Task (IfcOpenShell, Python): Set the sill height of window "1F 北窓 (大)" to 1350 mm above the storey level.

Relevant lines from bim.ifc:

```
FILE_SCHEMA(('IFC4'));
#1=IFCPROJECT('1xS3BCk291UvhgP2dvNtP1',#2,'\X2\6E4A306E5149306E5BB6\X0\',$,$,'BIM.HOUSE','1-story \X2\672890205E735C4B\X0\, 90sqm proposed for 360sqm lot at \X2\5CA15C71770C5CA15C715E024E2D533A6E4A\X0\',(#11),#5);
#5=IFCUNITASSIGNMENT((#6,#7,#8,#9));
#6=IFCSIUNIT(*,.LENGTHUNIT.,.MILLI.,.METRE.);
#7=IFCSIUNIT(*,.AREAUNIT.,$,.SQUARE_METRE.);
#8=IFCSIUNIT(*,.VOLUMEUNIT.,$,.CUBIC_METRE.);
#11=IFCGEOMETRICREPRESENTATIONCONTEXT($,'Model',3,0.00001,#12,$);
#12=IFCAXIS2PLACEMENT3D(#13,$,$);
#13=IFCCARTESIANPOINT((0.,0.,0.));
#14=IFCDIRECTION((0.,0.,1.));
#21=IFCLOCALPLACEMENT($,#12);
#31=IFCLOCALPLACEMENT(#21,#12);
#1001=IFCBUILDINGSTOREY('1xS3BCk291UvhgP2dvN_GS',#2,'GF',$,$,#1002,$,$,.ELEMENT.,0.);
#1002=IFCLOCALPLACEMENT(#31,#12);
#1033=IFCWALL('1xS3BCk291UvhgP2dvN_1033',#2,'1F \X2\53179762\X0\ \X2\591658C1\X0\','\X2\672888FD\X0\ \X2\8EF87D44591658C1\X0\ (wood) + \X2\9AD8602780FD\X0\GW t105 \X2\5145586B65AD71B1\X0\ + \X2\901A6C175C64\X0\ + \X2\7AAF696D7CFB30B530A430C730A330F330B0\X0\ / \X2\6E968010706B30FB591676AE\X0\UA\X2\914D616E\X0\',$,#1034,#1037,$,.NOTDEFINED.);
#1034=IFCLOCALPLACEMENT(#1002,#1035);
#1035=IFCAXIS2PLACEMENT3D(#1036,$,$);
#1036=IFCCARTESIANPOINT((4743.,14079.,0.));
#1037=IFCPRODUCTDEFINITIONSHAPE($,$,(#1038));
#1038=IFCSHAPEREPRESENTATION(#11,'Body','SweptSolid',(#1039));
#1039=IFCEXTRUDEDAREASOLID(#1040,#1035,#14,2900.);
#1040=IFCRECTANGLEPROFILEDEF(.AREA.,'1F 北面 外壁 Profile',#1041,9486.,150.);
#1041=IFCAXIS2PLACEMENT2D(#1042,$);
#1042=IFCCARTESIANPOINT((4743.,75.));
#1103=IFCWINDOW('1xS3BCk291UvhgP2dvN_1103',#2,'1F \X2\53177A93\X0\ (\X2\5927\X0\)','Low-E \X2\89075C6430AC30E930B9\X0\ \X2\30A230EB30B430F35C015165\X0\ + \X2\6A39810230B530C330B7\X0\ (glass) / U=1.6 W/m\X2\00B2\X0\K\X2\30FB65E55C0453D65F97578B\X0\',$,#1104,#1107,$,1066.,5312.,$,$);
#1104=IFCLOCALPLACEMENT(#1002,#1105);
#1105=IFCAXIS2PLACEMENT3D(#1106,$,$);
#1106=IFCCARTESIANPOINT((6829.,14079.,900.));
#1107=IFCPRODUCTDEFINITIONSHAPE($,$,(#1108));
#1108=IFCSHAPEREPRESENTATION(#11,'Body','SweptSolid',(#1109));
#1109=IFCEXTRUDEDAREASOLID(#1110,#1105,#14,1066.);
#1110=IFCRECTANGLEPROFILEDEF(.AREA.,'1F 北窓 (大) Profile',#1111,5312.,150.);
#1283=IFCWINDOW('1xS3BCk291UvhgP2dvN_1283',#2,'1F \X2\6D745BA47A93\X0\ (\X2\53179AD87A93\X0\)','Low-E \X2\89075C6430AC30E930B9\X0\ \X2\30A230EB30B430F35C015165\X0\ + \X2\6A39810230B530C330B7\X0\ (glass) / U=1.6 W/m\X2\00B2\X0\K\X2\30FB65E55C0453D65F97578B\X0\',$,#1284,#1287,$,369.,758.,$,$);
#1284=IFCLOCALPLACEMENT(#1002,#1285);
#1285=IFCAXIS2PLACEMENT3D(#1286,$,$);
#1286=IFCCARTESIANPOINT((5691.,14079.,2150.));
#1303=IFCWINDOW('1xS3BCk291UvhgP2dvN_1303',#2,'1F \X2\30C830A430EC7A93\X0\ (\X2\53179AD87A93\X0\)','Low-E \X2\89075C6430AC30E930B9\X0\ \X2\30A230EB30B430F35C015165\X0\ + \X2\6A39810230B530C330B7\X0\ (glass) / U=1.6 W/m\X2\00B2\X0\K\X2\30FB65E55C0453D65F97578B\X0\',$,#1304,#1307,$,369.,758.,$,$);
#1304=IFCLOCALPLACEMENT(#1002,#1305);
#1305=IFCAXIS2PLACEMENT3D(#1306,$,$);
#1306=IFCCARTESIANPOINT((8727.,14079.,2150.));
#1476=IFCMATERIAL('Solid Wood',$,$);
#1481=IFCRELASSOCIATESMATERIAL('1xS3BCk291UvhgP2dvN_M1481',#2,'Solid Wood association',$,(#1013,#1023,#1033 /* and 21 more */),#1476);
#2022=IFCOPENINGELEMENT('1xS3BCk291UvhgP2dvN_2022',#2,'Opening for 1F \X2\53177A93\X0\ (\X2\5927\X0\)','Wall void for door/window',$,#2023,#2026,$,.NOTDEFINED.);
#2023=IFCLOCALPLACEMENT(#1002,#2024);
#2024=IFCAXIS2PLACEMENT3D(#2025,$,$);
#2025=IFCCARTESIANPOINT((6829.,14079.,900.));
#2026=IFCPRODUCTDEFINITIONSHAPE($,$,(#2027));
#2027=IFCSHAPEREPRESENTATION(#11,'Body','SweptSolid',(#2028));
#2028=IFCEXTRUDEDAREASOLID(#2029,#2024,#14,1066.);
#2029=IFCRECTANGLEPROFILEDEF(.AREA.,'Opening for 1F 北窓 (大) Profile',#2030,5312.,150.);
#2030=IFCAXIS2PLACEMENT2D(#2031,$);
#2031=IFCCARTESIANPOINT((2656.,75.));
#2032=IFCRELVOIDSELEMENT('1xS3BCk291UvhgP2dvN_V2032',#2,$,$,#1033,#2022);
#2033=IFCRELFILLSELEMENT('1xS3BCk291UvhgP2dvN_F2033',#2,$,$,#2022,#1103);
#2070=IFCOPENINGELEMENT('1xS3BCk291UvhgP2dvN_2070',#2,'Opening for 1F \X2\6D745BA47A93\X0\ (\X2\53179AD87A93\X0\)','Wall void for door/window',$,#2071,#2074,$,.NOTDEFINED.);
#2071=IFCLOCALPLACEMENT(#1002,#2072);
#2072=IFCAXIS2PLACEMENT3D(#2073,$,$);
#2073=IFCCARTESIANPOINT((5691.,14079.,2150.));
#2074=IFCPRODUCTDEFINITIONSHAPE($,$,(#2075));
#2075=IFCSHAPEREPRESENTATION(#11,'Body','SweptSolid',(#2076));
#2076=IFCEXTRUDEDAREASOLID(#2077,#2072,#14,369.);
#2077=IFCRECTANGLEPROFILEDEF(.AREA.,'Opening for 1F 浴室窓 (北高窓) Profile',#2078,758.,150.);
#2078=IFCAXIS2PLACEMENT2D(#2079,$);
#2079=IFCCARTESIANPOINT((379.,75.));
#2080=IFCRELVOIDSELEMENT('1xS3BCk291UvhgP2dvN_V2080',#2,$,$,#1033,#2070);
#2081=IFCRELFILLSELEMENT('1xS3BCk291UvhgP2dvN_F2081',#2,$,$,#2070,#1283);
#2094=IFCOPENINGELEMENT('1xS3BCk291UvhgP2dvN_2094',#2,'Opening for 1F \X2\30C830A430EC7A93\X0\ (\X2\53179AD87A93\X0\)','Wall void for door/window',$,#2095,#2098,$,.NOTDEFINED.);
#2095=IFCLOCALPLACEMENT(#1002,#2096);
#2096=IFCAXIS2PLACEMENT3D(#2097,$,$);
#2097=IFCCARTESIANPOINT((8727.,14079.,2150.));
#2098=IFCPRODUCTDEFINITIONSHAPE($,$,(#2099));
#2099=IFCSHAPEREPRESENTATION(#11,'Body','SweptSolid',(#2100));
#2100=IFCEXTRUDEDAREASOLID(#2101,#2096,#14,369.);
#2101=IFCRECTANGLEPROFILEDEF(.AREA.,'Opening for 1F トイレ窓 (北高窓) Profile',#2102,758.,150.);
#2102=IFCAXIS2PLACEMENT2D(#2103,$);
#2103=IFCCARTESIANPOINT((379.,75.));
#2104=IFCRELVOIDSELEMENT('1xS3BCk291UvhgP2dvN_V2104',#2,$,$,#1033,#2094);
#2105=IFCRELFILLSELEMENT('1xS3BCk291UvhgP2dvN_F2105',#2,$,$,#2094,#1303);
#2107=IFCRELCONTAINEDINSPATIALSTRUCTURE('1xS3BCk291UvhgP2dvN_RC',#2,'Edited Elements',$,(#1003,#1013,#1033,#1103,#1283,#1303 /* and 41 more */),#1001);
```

```python
import numpy as np
import ifcopenshell
import ifcopenshell.api.geometry
import ifcopenshell.geom
import ifcopenshell.util.element
import ifcopenshell.util.placement
import ifcopenshell.util.shape
import ifcopenshell.util.unit

model = ifcopenshell.open("bim.ifc")
unit_scale = ifcopenshell.util.unit.calculate_unit_scale(model)

window = model.by_guid("1xS3BCk291UvhgP2dvN_1103")
opening = window.FillsVoids[0].RelatingOpeningElement
storey = ifcopenshell.util.element.get_container(window, ifc_class="IfcBuildingStorey")
level = ifcopenshell.util.placement.get_local_placement(storey.ObjectPlacement)[2, 3]

# The opening's origin need not be at the sill, so measure its lowest point.
shape = ifcopenshell.geom.create_shape(ifcopenshell.geom.settings(), opening)
bottom = ifcopenshell.util.shape.get_shape_bottom_elevation(shape, shape.geometry) / unit_scale
dz = level + 1.35 / unit_scale - bottom

shift = np.array([0.0, 0.0, dz])
# The window is not placed relative to its opening, so move both.
for product in (opening, window):
    matrix = ifcopenshell.util.placement.get_local_placement(product.ObjectPlacement)
    matrix[:3, 3] += shift
    ifcopenshell.api.geometry.edit_object_placement(model, product=product, matrix=matrix, is_si=False)

print(f"moved by {dz * unit_scale:+.3f} m")

model.write("bim_v2.ifc")
```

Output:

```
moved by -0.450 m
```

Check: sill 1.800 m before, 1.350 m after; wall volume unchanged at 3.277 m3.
